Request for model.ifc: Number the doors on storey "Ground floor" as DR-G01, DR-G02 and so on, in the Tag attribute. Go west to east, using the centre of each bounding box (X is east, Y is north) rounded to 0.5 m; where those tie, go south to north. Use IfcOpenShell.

First a look at what the model holds.

```python
import ifcopenshell
import ifcopenshell.util.element
import ifcopenshell.util.placement

model = ifcopenshell.open("model.ifc")
print(model.schema)
storey = next(s for s in model.by_type("IfcBuildingStorey") if s.Name == "Ground floor")
doors = [e for e in ifcopenshell.util.element.get_decomposition(storey) if e.is_a("IfcDoor")]
for e in sorted(doors, key=lambda e: e.id()):
    origin = ifcopenshell.util.placement.get_local_placement(e.ObjectPlacement)[:3, 3]
    print(e.id(), e.Tag, e.Name, origin.round(2) + 0.0, sep=" | ")
```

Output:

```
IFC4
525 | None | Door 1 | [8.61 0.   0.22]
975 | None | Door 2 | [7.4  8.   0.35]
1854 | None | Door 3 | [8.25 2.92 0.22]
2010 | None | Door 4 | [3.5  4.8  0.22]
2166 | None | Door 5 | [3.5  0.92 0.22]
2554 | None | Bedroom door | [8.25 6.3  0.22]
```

```python
import ifcopenshell
import ifcopenshell.geom
import ifcopenshell.util.element
import ifcopenshell.util.shape

model = ifcopenshell.open("model.ifc")
settings = ifcopenshell.geom.settings()
settings.set("use-world-coords", True)


def centre(element):
    shape = ifcopenshell.geom.create_shape(settings, element)
    return ifcopenshell.util.shape.get_bbox_centroid(shape.geometry)


storey = next(s for s in model.by_type("IfcBuildingStorey") if s.Name == "Ground floor")
doors = [e for e in ifcopenshell.util.element.get_decomposition(storey) if e.is_a("IfcDoor")]

# Insertion points can sit at a corner or the storey origin, so sort by the geometry (in metres).
centres = {e: centre(e) for e in doors}
doors.sort(key=lambda e: (round(centres[e][0] / 0.5), centres[e][1]))

for i, e in enumerate(doors, start=1):
    number = f"DR-G{i:02d}"
    e.Tag = number
    print(e.id(), number)

model.write("model_rev.ifc")
```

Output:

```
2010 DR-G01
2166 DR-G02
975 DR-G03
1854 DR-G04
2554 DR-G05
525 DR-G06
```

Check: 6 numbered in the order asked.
